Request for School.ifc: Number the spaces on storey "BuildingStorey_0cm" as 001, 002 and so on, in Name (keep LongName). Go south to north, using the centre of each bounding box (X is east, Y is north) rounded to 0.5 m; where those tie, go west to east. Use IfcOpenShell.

First a look at what the model holds.

```python
import ifcopenshell
import ifcopenshell.util.element
import ifcopenshell.util.placement

model = ifcopenshell.open("School.ifc")
print(model.schema)
storey = next(s for s in model.by_type("IfcBuildingStorey") if s.Name == "BuildingStorey_0cm")
spaces = [e for e in ifcopenshell.util.element.get_decomposition(storey) if e.is_a("IfcSpace")]
for e in sorted(spaces, key=lambda e: e.id()):
    origin = ifcopenshell.util.placement.get_local_placement(e.ObjectPlacement)[:3, 3]
    print(e.id(), e.Name, e.LongName, origin.round(2) + 0.0, sep=" | ")
```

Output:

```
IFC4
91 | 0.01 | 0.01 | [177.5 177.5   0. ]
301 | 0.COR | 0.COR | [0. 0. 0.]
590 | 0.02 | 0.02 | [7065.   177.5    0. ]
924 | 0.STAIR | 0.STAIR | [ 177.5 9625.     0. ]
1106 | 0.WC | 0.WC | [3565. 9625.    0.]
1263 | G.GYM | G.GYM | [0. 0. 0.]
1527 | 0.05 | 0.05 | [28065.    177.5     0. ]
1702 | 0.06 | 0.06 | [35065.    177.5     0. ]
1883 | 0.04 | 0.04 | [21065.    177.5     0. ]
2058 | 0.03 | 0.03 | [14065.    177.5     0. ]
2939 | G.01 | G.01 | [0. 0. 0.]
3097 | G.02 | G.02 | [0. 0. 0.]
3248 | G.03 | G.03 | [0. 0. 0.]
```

```python
import ifcopenshell
import ifcopenshell.geom
import ifcopenshell.util.element
import ifcopenshell.util.shape

model = ifcopenshell.open("School.ifc")
settings = ifcopenshell.geom.settings()
settings.set("use-world-coords", True)


def centre(element):
    shape = ifcopenshell.geom.create_shape(settings, element)
    return ifcopenshell.util.shape.get_bbox_centroid(shape.geometry)


storey = next(s for s in model.by_type("IfcBuildingStorey") if s.Name == "BuildingStorey_0cm")
spaces = [e for e in ifcopenshell.util.element.get_decomposition(storey) if e.is_a("IfcSpace")]

# Insertion points can sit at a corner or the storey origin, so sort by the geometry (in metres).
centres = {e: centre(e) for e in spaces}
spaces.sort(key=lambda e: (round(centres[e][1] / 0.5), centres[e][0]))

for i, e in enumerate(spaces, start=1):
    number = f"0{i:02d}"
    e.Name = number
    print(e.id(), number)

model.write("School_updated.ifc")
```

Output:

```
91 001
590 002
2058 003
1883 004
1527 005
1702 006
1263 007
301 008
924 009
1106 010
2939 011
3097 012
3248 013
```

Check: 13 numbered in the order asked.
